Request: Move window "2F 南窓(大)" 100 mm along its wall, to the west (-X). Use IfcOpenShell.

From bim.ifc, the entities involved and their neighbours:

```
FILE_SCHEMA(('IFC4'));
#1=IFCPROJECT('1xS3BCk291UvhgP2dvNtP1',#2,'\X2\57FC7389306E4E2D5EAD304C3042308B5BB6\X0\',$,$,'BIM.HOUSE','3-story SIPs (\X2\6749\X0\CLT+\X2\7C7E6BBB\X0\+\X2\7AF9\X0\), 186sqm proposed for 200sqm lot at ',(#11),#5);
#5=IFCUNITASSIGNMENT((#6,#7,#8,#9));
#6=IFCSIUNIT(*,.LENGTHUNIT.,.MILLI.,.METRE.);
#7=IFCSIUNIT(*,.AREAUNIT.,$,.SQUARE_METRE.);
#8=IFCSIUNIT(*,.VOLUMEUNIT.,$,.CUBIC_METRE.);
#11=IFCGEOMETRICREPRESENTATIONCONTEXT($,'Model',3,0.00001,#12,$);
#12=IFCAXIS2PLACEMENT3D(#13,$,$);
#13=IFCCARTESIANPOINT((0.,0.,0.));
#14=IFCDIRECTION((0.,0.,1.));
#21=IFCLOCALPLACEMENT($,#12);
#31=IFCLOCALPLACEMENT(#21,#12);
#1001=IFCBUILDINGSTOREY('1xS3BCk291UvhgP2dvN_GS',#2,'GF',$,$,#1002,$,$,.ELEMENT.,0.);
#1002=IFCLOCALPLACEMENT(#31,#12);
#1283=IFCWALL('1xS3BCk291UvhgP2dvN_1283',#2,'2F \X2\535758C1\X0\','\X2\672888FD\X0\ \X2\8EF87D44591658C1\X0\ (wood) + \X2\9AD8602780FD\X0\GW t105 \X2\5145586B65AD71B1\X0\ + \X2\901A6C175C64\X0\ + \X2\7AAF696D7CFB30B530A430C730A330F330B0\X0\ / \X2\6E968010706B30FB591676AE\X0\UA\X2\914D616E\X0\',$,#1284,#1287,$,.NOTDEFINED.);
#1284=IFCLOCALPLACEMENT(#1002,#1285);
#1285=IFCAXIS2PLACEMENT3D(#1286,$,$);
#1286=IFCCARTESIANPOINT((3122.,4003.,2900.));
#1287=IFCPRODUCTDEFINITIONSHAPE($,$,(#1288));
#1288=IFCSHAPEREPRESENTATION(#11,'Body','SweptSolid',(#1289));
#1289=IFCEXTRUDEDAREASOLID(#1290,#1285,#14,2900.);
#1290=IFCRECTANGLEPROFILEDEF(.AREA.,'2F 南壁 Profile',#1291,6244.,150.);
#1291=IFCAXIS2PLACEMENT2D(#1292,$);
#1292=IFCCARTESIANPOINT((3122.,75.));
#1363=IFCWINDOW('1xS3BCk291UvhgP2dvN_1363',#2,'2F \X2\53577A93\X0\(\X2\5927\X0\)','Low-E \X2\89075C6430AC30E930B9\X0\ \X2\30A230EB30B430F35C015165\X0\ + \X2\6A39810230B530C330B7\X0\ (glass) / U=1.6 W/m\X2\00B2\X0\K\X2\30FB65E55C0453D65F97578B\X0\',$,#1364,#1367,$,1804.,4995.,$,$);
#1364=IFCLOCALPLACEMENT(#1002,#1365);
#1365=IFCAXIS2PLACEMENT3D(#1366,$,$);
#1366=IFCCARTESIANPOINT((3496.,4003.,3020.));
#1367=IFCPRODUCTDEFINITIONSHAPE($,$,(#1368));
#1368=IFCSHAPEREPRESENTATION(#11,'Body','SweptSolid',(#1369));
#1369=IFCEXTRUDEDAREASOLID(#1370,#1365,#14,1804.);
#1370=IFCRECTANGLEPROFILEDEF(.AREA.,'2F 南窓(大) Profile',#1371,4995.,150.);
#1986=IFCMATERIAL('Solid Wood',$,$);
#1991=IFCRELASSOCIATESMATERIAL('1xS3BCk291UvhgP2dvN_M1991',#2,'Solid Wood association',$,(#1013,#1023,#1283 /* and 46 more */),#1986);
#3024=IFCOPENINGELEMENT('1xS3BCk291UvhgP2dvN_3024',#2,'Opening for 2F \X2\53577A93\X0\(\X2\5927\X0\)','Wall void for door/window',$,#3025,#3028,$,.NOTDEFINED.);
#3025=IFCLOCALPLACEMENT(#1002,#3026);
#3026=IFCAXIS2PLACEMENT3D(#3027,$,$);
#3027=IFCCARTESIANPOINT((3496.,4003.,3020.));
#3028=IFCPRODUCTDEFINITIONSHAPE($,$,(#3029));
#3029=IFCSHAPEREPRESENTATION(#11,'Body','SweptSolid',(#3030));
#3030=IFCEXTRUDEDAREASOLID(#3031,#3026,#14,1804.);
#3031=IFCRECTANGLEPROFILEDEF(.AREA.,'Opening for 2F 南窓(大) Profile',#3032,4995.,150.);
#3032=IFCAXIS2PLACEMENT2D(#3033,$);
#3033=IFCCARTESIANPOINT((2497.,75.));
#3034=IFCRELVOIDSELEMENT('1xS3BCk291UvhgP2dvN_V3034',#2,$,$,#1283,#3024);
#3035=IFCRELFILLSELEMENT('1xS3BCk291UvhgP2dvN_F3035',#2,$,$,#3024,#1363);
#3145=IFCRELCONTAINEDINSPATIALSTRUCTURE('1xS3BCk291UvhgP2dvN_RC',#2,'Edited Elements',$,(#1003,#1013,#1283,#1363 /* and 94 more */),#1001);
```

```python
import ifcopenshell
import ifcopenshell.api.geometry
import ifcopenshell.util.placement

model = ifcopenshell.open("bim.ifc")

window = model.by_id(1363)
opening = window.FillsVoids[0].RelatingOpeningElement
wall = opening.VoidsElements[0].RelatingBuildingElement

wall_matrix = ifcopenshell.util.placement.get_local_placement(wall.ObjectPlacement)
shift = wall_matrix[:3, 0] * -100.0
before = ifcopenshell.util.placement.get_local_placement(window.ObjectPlacement)[:3, 3].copy()

# The window is not placed relative to its opening, so move both.
for product in (opening, window):
    matrix = ifcopenshell.util.placement.get_local_placement(product.ObjectPlacement)
    matrix[:3, 3] += shift
    ifcopenshell.api.geometry.edit_object_placement(model, product=product, matrix=matrix, is_si=False)

after = ifcopenshell.util.placement.get_local_placement(window.ObjectPlacement)[:3, 3]
print("window moved by", (after - before).round(3) + 0.0)

model.write("bim-out.ifc")
```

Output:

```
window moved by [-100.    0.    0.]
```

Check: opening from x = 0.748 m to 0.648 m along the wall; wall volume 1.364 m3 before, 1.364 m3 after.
